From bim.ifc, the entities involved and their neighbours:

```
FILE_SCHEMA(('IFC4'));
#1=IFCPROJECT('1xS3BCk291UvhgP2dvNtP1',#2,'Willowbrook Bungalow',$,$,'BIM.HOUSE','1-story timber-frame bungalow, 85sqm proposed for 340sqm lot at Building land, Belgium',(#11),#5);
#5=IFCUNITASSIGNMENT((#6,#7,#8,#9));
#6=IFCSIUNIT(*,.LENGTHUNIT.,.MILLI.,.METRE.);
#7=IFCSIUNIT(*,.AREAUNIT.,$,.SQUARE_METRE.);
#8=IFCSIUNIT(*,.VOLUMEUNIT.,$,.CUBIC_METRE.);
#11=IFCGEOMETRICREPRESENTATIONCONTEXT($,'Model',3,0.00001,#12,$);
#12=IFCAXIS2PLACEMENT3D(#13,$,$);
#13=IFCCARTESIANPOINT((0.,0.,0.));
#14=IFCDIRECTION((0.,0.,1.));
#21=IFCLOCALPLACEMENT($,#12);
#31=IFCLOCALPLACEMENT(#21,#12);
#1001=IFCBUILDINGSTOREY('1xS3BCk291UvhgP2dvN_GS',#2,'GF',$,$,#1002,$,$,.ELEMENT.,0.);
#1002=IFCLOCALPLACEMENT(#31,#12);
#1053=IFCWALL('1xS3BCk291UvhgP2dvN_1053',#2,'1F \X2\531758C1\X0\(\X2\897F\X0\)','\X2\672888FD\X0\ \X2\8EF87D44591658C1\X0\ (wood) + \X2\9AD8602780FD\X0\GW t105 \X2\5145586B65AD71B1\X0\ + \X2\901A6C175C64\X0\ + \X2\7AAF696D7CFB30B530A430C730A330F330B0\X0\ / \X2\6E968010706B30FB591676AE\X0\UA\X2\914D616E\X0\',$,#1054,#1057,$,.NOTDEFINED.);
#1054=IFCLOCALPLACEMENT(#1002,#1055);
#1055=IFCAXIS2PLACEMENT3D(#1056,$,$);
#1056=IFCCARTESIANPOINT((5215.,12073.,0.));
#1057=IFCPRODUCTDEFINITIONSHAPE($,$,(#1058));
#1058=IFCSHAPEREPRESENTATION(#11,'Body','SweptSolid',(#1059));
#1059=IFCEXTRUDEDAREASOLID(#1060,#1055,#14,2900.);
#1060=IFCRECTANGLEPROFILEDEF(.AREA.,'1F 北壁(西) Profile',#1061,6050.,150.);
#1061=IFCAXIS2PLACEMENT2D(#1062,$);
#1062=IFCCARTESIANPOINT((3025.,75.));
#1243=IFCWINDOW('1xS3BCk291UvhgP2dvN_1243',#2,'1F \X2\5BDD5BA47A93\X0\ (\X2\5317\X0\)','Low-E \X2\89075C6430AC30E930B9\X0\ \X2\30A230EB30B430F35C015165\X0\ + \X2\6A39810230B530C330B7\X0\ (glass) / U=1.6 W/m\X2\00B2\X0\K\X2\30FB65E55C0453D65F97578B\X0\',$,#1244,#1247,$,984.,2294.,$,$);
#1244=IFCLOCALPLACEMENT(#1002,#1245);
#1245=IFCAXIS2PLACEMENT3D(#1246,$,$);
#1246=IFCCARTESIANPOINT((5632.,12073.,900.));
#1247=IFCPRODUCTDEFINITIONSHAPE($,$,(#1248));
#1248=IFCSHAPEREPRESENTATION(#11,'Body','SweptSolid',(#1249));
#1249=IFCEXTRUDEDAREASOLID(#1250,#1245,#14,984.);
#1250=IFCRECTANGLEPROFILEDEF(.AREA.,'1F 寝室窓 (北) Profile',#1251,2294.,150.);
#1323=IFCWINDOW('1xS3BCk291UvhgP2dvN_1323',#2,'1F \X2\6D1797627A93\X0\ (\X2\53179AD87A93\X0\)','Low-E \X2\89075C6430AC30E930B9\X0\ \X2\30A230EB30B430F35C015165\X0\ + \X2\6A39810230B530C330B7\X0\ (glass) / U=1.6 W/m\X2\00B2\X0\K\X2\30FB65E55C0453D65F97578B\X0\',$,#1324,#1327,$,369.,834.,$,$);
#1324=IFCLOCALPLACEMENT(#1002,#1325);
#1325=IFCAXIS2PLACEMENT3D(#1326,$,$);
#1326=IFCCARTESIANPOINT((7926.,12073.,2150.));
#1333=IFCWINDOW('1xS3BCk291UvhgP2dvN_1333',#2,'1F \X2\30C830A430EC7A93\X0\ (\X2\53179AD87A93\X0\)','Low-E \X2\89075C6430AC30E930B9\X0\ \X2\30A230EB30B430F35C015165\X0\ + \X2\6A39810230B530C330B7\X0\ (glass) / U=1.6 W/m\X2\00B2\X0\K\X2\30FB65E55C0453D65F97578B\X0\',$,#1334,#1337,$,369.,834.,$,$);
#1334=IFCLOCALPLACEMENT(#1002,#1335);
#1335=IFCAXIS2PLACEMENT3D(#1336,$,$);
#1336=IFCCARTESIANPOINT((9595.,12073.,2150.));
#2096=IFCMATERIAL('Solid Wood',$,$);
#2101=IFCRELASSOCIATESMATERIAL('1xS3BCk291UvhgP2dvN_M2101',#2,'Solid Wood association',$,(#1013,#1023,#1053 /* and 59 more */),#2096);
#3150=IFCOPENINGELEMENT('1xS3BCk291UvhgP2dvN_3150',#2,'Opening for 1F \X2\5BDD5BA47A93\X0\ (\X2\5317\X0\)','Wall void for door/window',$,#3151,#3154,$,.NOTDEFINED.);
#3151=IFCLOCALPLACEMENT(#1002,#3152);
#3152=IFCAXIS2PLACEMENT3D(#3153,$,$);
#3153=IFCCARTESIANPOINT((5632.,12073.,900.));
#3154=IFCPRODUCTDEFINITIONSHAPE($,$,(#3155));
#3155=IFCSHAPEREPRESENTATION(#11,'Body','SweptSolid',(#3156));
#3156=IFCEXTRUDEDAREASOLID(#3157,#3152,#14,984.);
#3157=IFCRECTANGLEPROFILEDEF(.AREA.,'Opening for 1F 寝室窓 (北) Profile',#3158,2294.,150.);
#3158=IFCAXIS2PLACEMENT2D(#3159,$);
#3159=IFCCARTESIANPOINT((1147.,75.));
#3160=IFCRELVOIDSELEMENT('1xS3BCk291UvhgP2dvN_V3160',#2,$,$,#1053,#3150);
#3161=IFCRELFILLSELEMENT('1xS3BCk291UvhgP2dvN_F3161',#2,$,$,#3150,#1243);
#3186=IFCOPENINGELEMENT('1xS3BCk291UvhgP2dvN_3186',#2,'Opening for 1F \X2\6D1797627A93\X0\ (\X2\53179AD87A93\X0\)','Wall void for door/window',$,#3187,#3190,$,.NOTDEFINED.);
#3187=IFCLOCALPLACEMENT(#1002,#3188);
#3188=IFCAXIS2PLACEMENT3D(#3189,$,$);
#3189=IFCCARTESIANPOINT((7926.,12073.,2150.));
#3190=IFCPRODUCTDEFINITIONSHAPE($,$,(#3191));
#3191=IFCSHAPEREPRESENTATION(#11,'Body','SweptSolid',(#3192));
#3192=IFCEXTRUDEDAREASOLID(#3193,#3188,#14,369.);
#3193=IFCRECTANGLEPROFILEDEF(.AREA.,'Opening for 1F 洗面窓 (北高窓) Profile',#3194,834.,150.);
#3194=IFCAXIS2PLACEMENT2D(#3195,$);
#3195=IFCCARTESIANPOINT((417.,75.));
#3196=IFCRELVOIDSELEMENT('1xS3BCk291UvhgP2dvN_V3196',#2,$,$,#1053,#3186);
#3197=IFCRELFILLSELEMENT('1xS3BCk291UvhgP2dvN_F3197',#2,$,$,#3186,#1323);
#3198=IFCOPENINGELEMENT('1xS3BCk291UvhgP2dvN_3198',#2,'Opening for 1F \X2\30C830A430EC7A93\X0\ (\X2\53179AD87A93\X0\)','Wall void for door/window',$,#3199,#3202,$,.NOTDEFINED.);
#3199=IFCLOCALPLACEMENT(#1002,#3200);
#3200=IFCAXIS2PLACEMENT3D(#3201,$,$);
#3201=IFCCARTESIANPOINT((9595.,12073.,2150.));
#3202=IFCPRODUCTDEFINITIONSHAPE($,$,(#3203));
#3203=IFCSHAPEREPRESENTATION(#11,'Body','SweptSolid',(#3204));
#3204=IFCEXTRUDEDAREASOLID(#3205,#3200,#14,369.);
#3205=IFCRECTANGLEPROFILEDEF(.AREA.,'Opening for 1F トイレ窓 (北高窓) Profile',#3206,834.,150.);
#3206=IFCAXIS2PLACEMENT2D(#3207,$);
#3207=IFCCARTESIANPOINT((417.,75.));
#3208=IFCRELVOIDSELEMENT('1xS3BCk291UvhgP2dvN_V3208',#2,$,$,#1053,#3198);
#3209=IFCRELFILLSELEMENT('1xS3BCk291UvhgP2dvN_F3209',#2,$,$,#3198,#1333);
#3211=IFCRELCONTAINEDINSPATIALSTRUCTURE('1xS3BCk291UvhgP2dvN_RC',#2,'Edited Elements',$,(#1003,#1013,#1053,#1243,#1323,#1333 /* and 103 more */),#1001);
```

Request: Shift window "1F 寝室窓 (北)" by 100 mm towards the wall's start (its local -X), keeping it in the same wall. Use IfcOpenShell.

```python
import ifcopenshell
import ifcopenshell.api.geometry
import ifcopenshell.util.placement
import ifcopenshell.util.unit

model = ifcopenshell.open("bim.ifc")
unit_scale = ifcopenshell.util.unit.calculate_unit_scale(model)

window = model.by_id(1243)
opening = window.FillsVoids[0].RelatingOpeningElement
wall = opening.VoidsElements[0].RelatingBuildingElement

wall_matrix = ifcopenshell.util.placement.get_local_placement(wall.ObjectPlacement)
shift = wall_matrix[:3, 0] * -0.1 / unit_scale
before = ifcopenshell.util.placement.get_local_placement(window.ObjectPlacement)[:3, 3].copy()

# The window is not placed relative to its opening, so move both.
for product in (opening, window):
    matrix = ifcopenshell.util.placement.get_local_placement(product.ObjectPlacement)
    matrix[:3, 3] += shift
    ifcopenshell.api.geometry.edit_object_placement(model, product=product, matrix=matrix, is_si=False)

after = ifcopenshell.util.placement.get_local_placement(window.ObjectPlacement)[:3, 3]
print("window moved by", (after - before).round(3) + 0.0)

model.write("bim_v2.ifc")
```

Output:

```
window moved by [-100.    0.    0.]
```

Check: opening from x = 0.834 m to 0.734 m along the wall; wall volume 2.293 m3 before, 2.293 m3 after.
